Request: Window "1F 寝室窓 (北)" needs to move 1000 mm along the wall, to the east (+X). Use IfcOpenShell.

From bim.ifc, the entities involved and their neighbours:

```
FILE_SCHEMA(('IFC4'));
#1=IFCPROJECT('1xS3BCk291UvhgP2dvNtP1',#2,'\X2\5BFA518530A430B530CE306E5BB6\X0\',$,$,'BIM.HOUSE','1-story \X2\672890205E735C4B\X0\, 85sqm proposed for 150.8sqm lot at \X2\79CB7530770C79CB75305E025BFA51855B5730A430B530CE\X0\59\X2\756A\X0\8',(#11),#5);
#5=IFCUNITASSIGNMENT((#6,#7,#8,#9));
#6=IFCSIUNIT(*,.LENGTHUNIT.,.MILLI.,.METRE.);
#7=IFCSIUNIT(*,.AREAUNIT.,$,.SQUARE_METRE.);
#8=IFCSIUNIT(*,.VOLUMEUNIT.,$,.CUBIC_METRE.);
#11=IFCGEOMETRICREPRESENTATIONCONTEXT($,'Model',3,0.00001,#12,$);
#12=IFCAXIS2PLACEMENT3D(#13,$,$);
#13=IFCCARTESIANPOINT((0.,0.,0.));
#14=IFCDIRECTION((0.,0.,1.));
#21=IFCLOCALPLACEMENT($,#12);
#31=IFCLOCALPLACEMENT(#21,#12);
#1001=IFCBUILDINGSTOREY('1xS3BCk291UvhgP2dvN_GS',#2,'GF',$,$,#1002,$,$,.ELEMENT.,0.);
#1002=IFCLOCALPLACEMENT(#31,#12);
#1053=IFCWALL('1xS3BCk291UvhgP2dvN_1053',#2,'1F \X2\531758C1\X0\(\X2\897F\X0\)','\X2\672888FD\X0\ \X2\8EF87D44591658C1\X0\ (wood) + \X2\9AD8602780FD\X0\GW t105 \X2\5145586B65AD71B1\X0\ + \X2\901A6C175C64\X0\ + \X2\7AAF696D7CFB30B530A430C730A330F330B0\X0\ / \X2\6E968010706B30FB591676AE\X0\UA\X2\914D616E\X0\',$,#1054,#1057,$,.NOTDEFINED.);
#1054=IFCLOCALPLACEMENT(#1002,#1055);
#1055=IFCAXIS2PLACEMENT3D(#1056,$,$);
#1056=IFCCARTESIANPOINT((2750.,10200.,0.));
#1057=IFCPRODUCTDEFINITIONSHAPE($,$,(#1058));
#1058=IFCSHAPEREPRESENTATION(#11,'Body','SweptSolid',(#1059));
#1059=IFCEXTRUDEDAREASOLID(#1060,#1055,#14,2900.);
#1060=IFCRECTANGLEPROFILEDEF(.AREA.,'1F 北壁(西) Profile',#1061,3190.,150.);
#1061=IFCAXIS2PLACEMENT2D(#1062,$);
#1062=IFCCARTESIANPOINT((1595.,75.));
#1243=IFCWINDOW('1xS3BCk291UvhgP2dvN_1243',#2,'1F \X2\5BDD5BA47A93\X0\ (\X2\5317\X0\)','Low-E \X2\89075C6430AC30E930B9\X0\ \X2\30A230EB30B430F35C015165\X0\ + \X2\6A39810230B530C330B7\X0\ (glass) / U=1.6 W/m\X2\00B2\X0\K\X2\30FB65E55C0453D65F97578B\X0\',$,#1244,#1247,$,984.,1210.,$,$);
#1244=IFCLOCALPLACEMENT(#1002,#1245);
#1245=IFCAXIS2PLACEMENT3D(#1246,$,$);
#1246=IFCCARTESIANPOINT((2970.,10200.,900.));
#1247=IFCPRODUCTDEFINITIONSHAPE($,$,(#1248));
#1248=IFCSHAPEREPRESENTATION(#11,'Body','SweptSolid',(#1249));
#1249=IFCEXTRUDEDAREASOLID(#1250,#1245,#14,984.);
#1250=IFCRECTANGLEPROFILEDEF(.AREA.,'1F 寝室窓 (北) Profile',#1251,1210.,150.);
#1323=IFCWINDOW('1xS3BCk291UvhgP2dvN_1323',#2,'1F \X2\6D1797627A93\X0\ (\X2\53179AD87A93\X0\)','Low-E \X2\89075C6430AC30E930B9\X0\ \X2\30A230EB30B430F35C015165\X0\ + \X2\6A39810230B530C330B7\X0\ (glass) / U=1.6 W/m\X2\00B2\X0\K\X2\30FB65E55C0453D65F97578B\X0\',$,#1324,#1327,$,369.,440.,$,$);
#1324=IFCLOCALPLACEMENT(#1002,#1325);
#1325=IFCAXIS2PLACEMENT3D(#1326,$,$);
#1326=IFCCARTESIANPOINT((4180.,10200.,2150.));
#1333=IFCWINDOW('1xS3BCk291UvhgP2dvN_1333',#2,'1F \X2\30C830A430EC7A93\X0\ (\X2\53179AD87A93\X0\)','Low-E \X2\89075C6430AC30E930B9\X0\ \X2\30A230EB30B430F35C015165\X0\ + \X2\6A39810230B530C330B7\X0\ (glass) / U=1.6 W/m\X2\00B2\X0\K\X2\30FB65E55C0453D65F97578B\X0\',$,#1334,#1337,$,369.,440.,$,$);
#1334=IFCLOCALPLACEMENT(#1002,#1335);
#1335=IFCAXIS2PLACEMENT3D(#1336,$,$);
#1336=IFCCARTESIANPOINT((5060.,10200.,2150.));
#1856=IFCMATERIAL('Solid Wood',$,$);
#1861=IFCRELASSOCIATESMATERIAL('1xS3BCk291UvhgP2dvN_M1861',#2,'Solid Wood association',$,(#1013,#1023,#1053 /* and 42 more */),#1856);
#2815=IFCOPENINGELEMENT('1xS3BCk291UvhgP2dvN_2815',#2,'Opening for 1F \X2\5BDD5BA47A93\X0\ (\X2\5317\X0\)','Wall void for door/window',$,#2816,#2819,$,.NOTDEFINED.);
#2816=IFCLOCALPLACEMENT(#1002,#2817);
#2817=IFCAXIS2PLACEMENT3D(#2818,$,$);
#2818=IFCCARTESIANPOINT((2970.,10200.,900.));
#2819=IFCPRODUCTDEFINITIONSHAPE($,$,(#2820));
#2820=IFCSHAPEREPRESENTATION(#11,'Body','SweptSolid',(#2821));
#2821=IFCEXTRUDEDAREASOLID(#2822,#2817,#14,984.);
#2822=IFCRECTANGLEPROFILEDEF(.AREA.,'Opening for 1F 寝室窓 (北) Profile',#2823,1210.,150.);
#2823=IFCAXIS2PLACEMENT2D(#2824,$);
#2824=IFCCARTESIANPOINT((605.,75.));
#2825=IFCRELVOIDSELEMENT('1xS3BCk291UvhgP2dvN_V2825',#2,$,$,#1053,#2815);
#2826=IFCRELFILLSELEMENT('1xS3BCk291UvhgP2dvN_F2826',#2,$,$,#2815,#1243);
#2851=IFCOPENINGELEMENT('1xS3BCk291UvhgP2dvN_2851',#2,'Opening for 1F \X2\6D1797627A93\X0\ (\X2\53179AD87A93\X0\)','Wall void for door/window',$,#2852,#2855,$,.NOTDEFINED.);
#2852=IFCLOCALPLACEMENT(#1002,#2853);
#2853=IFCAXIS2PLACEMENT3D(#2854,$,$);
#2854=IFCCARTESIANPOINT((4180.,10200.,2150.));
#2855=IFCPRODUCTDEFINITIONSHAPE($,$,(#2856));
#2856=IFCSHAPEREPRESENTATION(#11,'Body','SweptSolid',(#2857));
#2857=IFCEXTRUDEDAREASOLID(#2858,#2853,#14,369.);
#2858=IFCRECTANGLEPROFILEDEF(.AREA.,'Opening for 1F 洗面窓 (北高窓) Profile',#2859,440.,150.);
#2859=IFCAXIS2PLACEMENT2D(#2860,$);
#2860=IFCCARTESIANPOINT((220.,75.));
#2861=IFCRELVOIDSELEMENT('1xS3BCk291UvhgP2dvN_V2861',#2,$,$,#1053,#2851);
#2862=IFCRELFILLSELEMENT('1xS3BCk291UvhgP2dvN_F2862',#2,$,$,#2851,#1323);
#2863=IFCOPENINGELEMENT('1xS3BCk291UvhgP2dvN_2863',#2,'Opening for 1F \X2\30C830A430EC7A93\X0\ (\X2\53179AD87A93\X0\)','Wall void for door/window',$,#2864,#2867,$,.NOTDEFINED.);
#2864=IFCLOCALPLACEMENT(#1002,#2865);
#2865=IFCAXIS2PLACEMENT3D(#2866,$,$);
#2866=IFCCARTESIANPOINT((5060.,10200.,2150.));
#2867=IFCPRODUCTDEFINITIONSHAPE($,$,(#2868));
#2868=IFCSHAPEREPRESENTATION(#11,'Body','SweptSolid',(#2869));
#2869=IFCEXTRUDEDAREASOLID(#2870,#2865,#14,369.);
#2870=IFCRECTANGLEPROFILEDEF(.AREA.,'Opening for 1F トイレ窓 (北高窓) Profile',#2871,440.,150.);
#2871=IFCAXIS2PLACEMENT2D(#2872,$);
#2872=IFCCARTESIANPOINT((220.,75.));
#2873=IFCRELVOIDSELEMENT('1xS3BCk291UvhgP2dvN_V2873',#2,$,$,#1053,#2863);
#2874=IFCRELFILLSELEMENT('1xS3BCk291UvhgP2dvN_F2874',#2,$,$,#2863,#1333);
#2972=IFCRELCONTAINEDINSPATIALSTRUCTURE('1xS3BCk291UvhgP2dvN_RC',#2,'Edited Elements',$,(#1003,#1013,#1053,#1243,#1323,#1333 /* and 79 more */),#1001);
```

```python
import ifcopenshell
import ifcopenshell.api.geometry
import ifcopenshell.util.placement
import ifcopenshell.util.unit

model = ifcopenshell.open("bim.ifc")
unit_scale = ifcopenshell.util.unit.calculate_unit_scale(model)

window = model.by_id(1243)
opening = window.FillsVoids[0].RelatingOpeningElement
wall = opening.VoidsElements[0].RelatingBuildingElement

wall_matrix = ifcopenshell.util.placement.get_local_placement(wall.ObjectPlacement)
shift = wall_matrix[:3, 0] * 1 / unit_scale
before = ifcopenshell.util.placement.get_local_placement(window.ObjectPlacement)[:3, 3].copy()

# The window is not placed relative to its opening, so move both.
for product in (opening, window):
    matrix = ifcopenshell.util.placement.get_local_placement(product.ObjectPlacement)
    matrix[:3, 3] += shift
    ifcopenshell.api.geometry.edit_object_placement(model, product=product, matrix=matrix, is_si=False)

after = ifcopenshell.util.placement.get_local_placement(window.ObjectPlacement)[:3, 3]
print("window moved by", (after - before).round(3) + 0.0)

model.write("bim_v2.ifc")
```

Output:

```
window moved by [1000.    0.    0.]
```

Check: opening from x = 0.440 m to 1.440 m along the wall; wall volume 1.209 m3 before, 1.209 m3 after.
